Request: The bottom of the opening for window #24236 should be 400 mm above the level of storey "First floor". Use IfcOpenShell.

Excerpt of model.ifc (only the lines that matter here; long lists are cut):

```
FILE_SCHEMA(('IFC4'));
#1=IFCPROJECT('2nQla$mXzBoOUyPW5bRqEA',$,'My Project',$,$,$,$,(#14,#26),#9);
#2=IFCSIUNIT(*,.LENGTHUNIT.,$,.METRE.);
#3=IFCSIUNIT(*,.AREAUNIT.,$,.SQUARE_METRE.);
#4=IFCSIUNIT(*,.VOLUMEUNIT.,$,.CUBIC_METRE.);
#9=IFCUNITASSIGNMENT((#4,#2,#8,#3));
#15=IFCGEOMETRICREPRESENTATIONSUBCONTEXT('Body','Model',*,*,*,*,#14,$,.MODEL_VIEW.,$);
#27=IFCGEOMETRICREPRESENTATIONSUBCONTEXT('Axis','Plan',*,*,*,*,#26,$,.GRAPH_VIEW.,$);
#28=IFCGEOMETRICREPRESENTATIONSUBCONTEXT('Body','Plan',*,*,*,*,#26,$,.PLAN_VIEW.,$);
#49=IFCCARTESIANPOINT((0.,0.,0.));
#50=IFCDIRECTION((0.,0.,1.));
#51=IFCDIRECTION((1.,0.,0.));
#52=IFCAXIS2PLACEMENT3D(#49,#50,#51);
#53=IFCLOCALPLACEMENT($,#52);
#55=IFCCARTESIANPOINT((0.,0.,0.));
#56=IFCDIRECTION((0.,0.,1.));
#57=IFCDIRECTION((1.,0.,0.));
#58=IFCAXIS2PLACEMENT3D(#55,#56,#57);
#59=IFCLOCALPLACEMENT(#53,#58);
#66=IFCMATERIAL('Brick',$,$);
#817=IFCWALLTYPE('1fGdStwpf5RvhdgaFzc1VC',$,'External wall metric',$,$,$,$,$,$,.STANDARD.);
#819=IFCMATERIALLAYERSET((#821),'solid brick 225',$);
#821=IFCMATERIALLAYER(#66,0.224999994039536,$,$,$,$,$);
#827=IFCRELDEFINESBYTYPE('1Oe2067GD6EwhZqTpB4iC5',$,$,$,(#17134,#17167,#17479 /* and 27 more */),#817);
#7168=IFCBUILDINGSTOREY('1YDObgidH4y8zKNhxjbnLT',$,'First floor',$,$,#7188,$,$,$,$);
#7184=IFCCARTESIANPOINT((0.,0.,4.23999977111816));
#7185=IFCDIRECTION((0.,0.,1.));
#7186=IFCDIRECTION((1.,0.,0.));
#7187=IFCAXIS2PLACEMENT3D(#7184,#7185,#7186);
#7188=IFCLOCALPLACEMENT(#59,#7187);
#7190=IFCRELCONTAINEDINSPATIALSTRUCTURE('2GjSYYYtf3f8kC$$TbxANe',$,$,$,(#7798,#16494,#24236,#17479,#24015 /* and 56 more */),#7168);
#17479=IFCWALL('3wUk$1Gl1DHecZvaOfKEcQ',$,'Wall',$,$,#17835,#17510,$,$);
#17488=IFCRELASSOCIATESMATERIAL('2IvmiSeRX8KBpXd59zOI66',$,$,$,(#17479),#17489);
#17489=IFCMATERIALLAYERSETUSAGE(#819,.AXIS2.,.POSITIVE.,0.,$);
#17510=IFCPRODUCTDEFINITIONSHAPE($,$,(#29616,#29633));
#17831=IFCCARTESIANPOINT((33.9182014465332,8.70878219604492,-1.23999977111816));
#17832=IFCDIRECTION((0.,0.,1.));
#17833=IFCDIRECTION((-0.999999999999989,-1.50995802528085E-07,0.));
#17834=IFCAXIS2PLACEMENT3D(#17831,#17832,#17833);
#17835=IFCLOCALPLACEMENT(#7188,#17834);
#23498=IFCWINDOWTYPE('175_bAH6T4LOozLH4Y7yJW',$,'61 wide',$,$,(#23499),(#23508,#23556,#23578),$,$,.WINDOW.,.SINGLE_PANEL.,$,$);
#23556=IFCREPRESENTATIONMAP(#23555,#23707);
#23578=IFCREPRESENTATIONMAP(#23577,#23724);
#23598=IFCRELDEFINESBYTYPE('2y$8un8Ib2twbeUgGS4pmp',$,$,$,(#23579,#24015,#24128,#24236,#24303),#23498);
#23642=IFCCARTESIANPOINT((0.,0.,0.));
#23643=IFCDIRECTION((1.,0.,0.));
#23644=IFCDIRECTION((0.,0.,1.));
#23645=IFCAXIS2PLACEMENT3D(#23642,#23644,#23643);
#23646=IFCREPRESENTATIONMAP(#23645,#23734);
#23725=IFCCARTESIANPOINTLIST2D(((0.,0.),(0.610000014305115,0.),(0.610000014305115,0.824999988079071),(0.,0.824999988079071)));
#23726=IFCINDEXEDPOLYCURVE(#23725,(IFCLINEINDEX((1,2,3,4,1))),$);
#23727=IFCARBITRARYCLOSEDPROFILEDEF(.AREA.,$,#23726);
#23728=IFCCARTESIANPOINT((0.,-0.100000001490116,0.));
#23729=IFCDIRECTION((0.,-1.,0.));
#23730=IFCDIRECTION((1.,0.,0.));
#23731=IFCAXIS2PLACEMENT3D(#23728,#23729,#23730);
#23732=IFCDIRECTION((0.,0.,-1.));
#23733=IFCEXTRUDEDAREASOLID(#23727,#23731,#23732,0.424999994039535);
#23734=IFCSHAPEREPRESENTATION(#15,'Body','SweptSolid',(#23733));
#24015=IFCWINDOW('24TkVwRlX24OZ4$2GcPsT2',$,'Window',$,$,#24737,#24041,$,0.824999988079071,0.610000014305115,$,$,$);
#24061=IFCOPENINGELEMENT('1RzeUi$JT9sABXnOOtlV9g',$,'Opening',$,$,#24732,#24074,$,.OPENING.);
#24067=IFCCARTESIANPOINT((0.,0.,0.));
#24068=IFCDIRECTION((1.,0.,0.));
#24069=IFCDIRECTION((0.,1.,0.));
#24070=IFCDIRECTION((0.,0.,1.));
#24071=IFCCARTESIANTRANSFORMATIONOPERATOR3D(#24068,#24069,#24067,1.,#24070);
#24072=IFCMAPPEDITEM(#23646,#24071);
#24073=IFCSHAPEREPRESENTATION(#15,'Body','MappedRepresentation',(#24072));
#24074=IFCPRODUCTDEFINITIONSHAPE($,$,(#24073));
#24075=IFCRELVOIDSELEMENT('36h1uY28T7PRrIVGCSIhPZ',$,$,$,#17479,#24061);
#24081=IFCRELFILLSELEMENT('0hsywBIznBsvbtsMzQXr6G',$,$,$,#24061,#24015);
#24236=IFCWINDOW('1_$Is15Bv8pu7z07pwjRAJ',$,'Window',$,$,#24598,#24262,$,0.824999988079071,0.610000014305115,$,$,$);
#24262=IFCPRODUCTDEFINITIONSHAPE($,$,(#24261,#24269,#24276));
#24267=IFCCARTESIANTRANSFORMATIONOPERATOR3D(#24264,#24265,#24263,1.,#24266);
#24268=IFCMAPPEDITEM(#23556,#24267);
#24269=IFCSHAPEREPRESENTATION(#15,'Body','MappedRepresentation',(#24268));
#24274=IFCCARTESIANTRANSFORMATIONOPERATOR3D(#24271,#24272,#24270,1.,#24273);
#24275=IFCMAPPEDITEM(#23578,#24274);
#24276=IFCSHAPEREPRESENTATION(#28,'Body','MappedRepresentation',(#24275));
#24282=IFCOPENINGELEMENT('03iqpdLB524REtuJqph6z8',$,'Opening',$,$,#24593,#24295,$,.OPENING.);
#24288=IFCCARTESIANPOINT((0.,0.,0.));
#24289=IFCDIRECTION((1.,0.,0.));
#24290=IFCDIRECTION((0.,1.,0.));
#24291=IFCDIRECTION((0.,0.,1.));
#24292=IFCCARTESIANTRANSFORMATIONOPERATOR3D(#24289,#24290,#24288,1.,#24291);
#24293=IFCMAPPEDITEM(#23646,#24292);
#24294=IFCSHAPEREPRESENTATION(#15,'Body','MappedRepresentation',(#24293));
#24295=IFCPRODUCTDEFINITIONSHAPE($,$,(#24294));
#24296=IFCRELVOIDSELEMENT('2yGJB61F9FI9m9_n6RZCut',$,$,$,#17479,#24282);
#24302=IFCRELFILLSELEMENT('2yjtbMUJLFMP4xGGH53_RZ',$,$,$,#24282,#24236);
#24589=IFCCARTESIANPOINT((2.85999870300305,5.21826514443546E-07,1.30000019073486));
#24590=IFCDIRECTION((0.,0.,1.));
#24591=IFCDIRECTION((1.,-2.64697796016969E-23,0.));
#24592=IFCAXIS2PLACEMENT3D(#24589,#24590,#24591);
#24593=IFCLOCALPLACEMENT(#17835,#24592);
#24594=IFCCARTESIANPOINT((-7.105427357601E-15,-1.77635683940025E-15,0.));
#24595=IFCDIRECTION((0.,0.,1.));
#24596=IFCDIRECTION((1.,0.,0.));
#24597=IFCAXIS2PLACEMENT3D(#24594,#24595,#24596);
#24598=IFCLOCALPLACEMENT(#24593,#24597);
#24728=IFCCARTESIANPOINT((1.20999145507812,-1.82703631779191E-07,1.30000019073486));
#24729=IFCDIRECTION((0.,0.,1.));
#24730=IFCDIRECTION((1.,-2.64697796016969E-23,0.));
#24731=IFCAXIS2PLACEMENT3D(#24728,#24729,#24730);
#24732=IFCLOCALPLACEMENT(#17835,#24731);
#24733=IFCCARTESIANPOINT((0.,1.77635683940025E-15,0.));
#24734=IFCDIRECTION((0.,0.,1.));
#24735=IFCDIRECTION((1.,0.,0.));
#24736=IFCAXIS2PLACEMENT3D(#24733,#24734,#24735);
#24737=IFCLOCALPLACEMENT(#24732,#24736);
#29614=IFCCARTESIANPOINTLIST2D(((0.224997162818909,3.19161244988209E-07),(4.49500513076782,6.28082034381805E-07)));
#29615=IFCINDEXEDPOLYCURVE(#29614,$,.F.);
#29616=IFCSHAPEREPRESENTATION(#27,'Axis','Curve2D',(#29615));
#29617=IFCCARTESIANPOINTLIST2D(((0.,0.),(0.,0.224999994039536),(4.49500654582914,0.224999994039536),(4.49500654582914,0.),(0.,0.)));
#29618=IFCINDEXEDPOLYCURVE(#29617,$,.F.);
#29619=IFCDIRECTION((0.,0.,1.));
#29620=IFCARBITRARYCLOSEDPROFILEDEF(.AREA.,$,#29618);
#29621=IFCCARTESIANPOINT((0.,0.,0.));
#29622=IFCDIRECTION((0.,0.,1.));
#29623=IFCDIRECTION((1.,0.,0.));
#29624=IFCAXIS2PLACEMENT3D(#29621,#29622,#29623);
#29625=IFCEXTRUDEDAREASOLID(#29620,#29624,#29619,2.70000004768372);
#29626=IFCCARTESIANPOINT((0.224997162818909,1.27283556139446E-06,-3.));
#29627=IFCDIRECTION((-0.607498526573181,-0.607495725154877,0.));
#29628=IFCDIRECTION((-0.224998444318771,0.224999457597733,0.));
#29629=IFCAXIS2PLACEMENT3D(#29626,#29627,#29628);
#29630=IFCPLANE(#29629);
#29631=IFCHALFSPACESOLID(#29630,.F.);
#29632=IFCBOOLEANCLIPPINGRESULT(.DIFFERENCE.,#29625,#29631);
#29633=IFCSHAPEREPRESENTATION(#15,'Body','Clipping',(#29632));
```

```python
import numpy as np
import ifcopenshell
import ifcopenshell.api.geometry
import ifcopenshell.geom
import ifcopenshell.util.element
import ifcopenshell.util.placement
import ifcopenshell.util.shape
import ifcopenshell.util.unit

model = ifcopenshell.open("model.ifc")
unit_scale = ifcopenshell.util.unit.calculate_unit_scale(model)

window = model.by_guid("1_$Is15Bv8pu7z07pwjRAJ")
opening = window.FillsVoids[0].RelatingOpeningElement
storey = ifcopenshell.util.element.get_container(window, ifc_class="IfcBuildingStorey")
level = ifcopenshell.util.placement.get_local_placement(storey.ObjectPlacement)[2, 3]

# The opening's origin need not be at the sill, so measure its lowest point.
shape = ifcopenshell.geom.create_shape(ifcopenshell.geom.settings(), opening)
bottom = ifcopenshell.util.shape.get_shape_bottom_elevation(shape, shape.geometry) / unit_scale
dz = level + 0.4 - bottom

shift = np.array([0.0, 0.0, dz])
# The window is placed relative to its opening, so it follows when the opening moves.
matrix = ifcopenshell.util.placement.get_local_placement(opening.ObjectPlacement)
matrix[:3, 3] += shift
ifcopenshell.api.geometry.edit_object_placement(
    model, product=opening, matrix=matrix, is_si=False, should_transform_children=True
)

print(f"moved by {dz * unit_scale:+.3f} m")

model.write("model_updated.ifc")
```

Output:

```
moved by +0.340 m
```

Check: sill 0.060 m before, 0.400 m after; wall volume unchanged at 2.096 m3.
